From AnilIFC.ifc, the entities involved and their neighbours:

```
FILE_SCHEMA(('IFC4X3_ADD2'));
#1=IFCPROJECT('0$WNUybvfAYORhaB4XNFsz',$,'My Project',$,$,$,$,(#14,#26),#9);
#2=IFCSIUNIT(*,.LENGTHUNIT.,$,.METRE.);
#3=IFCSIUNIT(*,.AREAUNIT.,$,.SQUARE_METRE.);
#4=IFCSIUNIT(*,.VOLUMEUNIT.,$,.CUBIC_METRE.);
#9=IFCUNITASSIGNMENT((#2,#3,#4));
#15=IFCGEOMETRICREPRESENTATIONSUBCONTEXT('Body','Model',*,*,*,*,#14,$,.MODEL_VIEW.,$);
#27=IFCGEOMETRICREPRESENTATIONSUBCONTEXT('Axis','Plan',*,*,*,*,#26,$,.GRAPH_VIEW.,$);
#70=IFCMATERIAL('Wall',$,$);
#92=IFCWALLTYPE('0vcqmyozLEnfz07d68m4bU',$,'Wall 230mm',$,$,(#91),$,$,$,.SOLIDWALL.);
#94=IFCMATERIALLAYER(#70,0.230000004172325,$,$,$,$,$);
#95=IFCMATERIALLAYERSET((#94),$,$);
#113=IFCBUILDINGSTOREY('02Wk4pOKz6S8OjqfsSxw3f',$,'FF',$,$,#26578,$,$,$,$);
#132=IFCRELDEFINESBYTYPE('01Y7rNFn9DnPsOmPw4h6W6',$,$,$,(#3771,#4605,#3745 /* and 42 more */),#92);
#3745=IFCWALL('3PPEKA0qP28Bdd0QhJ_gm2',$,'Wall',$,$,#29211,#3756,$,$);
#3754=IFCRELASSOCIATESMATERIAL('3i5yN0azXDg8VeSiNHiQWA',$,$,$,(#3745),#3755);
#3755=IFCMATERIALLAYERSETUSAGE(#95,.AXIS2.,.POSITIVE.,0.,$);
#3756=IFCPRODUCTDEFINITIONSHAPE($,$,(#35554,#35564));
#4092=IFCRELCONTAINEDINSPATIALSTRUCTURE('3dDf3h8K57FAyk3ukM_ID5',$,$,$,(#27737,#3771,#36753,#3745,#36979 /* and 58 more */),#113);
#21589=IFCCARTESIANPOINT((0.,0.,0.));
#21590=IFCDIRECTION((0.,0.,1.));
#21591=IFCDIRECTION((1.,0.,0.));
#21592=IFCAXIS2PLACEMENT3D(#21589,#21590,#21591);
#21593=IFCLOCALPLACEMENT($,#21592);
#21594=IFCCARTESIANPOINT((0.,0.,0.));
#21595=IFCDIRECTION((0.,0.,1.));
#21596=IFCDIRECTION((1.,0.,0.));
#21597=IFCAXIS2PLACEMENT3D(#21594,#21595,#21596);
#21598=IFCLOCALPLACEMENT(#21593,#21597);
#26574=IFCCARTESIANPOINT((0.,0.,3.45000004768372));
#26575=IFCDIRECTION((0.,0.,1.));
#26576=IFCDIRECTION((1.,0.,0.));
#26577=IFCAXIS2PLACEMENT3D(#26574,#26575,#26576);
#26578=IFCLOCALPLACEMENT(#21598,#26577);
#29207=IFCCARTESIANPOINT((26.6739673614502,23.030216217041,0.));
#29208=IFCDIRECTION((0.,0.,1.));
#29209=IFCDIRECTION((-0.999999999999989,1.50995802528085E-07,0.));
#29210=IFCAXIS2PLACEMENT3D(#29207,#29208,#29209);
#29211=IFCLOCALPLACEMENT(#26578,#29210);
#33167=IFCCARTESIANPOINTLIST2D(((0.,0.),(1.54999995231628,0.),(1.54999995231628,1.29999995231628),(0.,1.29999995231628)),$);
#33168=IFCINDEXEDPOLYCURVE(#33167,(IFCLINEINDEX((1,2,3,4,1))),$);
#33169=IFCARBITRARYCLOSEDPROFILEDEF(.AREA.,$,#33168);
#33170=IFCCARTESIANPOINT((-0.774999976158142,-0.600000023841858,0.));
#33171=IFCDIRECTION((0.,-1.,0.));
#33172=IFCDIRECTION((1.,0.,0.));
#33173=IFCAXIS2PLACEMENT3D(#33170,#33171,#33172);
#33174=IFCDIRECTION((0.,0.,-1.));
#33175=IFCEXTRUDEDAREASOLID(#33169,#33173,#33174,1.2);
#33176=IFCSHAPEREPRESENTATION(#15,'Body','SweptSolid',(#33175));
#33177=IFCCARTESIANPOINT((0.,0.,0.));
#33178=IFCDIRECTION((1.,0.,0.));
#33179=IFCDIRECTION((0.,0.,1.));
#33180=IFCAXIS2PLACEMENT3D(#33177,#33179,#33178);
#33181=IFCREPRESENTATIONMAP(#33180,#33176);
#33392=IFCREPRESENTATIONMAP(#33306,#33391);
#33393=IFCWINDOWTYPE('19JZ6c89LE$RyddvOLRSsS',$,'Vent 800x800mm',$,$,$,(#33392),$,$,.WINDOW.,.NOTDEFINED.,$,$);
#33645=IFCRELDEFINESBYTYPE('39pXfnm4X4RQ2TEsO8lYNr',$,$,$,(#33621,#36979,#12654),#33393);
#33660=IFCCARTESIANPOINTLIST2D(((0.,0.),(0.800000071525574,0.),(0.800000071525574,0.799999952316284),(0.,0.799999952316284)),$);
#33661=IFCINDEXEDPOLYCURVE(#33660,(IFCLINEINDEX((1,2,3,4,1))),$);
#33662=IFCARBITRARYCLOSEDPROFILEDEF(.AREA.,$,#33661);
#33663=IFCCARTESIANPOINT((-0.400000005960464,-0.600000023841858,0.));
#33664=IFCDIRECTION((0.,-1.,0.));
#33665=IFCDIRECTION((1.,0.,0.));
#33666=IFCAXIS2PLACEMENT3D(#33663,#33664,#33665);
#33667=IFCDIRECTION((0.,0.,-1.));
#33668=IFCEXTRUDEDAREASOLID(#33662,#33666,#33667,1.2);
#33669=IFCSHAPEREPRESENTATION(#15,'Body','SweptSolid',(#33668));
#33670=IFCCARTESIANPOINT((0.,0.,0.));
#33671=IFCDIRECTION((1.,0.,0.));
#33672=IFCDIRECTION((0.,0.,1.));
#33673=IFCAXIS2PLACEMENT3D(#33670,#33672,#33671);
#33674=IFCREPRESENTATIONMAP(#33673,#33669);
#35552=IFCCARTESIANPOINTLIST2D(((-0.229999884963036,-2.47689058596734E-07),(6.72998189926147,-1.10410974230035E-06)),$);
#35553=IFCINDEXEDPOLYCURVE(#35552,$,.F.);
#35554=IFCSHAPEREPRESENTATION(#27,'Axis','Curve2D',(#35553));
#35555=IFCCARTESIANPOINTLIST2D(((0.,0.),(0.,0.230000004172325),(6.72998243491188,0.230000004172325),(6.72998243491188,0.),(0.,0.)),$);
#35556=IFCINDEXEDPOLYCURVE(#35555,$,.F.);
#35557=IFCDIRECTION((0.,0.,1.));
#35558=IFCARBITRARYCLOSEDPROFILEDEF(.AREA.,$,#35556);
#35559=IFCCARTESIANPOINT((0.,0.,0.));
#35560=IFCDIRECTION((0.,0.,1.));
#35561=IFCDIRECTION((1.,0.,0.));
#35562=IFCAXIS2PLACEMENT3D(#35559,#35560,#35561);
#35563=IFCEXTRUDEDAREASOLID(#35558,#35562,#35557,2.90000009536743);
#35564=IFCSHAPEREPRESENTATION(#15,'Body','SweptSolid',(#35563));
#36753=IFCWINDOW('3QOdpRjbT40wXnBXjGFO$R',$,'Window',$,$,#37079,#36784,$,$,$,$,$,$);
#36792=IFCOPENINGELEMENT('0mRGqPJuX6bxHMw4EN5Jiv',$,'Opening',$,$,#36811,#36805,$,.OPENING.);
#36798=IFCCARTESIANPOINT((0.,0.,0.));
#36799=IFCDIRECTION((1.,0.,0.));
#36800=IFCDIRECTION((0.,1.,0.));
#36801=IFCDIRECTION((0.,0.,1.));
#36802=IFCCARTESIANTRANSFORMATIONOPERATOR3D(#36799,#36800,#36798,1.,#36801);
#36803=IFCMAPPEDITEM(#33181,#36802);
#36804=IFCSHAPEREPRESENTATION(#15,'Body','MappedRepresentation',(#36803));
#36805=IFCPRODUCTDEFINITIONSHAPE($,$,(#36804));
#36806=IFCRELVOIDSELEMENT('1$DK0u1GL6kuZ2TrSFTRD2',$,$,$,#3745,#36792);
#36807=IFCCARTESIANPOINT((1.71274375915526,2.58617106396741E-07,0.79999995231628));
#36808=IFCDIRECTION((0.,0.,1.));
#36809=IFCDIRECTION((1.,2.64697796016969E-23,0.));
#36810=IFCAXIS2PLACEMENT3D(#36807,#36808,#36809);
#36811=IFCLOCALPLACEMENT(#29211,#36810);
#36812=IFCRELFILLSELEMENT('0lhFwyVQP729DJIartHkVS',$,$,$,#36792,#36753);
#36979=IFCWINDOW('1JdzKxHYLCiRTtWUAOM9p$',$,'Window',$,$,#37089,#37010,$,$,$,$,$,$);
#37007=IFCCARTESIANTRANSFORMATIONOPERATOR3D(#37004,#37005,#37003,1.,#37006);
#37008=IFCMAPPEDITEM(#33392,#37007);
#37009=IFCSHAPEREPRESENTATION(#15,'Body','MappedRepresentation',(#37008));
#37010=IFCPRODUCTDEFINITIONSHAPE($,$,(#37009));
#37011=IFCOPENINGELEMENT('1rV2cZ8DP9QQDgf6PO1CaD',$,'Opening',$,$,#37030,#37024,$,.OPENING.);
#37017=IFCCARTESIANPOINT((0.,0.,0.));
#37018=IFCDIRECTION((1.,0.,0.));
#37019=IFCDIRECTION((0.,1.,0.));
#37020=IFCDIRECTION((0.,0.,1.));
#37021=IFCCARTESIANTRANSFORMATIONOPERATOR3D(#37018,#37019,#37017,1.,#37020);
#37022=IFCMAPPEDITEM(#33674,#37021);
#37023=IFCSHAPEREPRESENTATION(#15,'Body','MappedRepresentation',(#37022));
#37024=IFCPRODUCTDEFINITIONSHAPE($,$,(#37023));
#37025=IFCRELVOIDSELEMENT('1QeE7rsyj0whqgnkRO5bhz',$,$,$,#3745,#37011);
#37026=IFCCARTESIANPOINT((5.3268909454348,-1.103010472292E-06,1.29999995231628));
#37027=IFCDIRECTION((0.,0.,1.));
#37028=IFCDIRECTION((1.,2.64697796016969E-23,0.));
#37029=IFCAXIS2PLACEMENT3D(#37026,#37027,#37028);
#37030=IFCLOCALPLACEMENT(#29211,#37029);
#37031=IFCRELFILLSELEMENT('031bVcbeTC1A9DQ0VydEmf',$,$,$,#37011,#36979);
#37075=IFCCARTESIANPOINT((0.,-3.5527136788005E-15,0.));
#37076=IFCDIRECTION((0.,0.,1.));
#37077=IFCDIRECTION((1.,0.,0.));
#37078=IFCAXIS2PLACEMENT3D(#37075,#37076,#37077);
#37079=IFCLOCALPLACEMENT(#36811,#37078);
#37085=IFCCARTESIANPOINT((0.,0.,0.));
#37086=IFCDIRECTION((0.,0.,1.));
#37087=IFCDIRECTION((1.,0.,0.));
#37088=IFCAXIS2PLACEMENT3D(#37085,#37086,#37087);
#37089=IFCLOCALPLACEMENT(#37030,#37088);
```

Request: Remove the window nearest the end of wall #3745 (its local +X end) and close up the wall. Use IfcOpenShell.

```python
import ifcopenshell
import ifcopenshell.api.feature
import ifcopenshell.api.root
import ifcopenshell.geom
import ifcopenshell.util.shape

model = ifcopenshell.open("AnilIFC.ifc")
settings = ifcopenshell.geom.settings()


def volume(element):
    """Net volume in cubic metres, openings subtracted."""
    shape = ifcopenshell.geom.create_shape(settings, element)
    return ifcopenshell.util.shape.get_volume(shape.geometry)


window = model.by_guid("1JdzKxHYLCiRTtWUAOM9p$")
opening = window.FillsVoids[0].RelatingOpeningElement
wall = opening.VoidsElements[0].RelatingBuildingElement
before = volume(wall)

ifcopenshell.api.root.remove_product(model, product=window)
ifcopenshell.api.feature.remove_feature(model, feature=opening)

after = volume(wall)

print(f"wall volume {before:.3f} -> {after:.3f} m3")

model.write("AnilIFC_rev.ifc")
```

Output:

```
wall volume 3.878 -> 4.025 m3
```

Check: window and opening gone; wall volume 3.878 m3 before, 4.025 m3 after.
